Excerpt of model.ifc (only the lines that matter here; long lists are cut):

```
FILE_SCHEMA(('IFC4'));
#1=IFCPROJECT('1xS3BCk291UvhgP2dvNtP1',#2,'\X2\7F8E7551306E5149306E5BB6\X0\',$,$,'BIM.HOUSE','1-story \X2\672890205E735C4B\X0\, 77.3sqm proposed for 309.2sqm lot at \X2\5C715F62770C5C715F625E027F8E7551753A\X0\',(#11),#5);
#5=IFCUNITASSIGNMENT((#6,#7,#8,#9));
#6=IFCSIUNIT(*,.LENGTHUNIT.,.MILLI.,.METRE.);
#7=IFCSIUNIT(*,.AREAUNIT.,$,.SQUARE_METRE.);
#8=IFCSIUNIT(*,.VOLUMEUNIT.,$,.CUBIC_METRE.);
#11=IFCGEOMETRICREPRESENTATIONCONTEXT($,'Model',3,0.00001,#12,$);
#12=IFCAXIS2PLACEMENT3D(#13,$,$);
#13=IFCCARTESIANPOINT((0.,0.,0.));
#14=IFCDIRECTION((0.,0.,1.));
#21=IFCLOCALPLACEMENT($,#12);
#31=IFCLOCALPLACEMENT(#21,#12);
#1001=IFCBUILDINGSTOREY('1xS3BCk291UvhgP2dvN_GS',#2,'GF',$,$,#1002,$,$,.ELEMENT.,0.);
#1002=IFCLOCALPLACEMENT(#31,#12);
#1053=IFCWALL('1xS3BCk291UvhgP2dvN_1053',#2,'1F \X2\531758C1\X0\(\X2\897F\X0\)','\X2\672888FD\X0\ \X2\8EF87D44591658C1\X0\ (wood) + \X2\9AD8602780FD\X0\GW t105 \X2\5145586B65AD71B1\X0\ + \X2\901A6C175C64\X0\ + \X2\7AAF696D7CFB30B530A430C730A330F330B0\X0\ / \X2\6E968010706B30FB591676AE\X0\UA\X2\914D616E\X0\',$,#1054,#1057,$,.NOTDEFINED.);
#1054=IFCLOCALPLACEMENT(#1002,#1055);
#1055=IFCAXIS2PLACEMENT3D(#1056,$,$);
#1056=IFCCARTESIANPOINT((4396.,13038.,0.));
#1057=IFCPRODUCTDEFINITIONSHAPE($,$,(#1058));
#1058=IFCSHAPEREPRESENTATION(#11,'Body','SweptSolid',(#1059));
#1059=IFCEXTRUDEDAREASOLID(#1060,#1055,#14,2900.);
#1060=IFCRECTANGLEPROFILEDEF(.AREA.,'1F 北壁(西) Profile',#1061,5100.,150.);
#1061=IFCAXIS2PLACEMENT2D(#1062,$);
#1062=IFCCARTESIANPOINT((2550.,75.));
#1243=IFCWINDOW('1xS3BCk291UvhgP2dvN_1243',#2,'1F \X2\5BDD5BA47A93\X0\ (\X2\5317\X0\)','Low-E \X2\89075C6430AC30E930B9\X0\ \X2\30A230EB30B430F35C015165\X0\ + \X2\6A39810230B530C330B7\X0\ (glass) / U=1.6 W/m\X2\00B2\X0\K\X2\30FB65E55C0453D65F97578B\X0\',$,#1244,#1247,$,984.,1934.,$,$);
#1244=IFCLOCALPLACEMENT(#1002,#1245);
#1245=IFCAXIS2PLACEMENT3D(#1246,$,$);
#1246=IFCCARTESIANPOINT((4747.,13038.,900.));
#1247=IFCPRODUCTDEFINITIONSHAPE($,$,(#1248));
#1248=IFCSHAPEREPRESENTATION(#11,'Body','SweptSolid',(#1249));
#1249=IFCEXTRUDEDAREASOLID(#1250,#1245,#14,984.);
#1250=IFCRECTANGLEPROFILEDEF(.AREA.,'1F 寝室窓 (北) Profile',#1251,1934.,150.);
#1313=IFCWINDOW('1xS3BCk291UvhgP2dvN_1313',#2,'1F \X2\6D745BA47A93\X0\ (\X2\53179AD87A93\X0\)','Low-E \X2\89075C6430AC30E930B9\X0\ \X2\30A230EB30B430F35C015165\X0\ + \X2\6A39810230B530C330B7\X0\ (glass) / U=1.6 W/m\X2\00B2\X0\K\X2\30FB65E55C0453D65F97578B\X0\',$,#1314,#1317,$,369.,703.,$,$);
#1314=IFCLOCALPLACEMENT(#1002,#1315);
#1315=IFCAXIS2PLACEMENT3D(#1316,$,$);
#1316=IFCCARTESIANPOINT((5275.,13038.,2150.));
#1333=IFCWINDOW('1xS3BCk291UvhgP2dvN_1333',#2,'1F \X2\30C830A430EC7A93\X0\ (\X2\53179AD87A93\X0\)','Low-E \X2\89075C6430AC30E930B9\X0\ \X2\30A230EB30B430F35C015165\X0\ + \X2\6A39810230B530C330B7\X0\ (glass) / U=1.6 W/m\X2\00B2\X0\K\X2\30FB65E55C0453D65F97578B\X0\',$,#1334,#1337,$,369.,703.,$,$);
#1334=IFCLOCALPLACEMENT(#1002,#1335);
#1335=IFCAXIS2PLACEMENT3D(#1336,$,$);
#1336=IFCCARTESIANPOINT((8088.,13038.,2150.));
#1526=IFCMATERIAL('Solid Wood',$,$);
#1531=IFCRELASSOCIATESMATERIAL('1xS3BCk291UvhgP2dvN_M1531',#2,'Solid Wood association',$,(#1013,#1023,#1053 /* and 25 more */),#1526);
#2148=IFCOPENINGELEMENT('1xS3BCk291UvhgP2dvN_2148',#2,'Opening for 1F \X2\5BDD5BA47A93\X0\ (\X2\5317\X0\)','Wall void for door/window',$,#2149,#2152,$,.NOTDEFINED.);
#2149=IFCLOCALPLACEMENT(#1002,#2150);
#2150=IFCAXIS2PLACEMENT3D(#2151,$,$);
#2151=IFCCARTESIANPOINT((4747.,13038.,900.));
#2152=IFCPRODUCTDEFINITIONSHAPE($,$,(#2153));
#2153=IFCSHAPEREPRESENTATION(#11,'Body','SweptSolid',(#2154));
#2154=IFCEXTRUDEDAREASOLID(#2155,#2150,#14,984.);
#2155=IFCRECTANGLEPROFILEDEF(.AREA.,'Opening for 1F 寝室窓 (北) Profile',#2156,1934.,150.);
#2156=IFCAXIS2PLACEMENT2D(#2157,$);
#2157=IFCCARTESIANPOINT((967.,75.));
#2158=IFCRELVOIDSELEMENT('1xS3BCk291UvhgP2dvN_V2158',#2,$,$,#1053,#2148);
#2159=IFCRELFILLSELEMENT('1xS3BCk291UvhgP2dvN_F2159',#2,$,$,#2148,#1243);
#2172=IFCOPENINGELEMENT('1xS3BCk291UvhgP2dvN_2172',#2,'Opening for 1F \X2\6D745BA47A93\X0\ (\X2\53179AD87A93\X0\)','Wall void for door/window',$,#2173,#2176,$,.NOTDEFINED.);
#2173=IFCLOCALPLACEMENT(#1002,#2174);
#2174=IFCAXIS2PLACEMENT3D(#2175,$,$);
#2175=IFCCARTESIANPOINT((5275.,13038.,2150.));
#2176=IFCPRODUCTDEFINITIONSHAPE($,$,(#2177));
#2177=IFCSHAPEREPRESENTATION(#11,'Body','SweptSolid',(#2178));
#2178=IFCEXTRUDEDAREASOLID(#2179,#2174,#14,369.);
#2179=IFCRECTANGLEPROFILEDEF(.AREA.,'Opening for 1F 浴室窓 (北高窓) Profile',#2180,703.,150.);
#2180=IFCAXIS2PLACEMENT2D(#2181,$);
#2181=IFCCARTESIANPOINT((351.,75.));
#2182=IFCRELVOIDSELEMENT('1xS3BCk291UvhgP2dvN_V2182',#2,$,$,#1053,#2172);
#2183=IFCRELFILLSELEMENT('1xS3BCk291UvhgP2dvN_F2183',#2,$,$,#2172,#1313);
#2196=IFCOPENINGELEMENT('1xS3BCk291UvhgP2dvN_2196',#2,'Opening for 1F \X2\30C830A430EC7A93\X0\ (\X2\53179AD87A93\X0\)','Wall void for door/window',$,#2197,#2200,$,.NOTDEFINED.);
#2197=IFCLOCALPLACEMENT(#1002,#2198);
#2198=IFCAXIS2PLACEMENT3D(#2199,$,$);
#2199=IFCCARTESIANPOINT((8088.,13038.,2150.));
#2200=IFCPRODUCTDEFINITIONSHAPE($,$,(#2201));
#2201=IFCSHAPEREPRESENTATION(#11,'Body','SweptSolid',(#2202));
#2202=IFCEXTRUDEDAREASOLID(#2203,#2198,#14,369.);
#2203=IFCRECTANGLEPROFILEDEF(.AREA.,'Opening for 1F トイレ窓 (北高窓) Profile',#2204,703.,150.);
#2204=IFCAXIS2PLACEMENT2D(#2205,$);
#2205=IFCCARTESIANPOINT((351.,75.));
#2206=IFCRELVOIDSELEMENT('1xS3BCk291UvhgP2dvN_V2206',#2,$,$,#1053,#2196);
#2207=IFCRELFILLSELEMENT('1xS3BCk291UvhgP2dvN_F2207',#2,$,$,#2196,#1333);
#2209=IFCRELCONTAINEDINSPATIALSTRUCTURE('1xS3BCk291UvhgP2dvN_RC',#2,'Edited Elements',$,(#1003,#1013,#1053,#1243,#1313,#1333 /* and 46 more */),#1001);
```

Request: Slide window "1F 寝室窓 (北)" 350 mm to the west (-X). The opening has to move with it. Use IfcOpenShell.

```python
import ifcopenshell
import ifcopenshell.api.geometry
import ifcopenshell.util.placement

model = ifcopenshell.open("model.ifc")

window = model.by_guid("1xS3BCk291UvhgP2dvN_1243")
opening = window.FillsVoids[0].RelatingOpeningElement
wall = opening.VoidsElements[0].RelatingBuildingElement

wall_matrix = ifcopenshell.util.placement.get_local_placement(wall.ObjectPlacement)
shift = wall_matrix[:3, 0] * -350.0
before = ifcopenshell.util.placement.get_local_placement(window.ObjectPlacement)[:3, 3].copy()

# The window is not placed relative to its opening, so move both.
for product in (opening, window):
    matrix = ifcopenshell.util.placement.get_local_placement(product.ObjectPlacement)
    matrix[:3, 3] += shift
    ifcopenshell.api.geometry.edit_object_placement(model, product=product, matrix=matrix, is_si=False)

after = ifcopenshell.util.placement.get_local_placement(window.ObjectPlacement)[:3, 3]
print("window moved by", (after - before).round(3) + 0.0)

model.write("model_edited.ifc")
```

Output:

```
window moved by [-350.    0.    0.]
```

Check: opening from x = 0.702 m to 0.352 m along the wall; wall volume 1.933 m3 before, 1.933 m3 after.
